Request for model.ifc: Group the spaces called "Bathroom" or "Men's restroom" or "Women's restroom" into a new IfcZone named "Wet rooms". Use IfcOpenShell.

First a look at what the model holds.

```python
import ifcopenshell

model = ifcopenshell.open("model.ifc")
print(model.schema)
seen = {}
for space in model.by_type("IfcSpace"):
    seen[space.LongName] = seen.get(space.LongName, 0) + 1
for name, count in sorted(seen.items(), key=str):
    print(count, "x", name)
print("zones:", [z.Name for z in model.by_type("IfcZone")][:20])
```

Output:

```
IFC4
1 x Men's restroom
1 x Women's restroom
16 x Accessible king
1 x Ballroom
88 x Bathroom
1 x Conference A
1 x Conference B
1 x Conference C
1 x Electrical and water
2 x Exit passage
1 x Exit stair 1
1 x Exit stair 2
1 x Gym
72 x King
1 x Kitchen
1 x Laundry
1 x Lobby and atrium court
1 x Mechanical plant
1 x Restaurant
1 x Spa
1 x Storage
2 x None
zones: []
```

```python
import ifcopenshell
import ifcopenshell.api.group
import ifcopenshell.api.root

model = ifcopenshell.open("model.ifc")

names = {"Bathroom", "Men's restroom", "Women's restroom"}
spaces = [s for s in model.by_type("IfcSpace") if s.LongName in names]

zone = ifcopenshell.api.root.create_entity(model, ifc_class="IfcZone", name="Wet rooms")
ifcopenshell.api.group.assign_group(model, products=spaces, group=zone)
print(len(spaces), "spaces in", zone.Name)

model.write("model_v2.ifc")
```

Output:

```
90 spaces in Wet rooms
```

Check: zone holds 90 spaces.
